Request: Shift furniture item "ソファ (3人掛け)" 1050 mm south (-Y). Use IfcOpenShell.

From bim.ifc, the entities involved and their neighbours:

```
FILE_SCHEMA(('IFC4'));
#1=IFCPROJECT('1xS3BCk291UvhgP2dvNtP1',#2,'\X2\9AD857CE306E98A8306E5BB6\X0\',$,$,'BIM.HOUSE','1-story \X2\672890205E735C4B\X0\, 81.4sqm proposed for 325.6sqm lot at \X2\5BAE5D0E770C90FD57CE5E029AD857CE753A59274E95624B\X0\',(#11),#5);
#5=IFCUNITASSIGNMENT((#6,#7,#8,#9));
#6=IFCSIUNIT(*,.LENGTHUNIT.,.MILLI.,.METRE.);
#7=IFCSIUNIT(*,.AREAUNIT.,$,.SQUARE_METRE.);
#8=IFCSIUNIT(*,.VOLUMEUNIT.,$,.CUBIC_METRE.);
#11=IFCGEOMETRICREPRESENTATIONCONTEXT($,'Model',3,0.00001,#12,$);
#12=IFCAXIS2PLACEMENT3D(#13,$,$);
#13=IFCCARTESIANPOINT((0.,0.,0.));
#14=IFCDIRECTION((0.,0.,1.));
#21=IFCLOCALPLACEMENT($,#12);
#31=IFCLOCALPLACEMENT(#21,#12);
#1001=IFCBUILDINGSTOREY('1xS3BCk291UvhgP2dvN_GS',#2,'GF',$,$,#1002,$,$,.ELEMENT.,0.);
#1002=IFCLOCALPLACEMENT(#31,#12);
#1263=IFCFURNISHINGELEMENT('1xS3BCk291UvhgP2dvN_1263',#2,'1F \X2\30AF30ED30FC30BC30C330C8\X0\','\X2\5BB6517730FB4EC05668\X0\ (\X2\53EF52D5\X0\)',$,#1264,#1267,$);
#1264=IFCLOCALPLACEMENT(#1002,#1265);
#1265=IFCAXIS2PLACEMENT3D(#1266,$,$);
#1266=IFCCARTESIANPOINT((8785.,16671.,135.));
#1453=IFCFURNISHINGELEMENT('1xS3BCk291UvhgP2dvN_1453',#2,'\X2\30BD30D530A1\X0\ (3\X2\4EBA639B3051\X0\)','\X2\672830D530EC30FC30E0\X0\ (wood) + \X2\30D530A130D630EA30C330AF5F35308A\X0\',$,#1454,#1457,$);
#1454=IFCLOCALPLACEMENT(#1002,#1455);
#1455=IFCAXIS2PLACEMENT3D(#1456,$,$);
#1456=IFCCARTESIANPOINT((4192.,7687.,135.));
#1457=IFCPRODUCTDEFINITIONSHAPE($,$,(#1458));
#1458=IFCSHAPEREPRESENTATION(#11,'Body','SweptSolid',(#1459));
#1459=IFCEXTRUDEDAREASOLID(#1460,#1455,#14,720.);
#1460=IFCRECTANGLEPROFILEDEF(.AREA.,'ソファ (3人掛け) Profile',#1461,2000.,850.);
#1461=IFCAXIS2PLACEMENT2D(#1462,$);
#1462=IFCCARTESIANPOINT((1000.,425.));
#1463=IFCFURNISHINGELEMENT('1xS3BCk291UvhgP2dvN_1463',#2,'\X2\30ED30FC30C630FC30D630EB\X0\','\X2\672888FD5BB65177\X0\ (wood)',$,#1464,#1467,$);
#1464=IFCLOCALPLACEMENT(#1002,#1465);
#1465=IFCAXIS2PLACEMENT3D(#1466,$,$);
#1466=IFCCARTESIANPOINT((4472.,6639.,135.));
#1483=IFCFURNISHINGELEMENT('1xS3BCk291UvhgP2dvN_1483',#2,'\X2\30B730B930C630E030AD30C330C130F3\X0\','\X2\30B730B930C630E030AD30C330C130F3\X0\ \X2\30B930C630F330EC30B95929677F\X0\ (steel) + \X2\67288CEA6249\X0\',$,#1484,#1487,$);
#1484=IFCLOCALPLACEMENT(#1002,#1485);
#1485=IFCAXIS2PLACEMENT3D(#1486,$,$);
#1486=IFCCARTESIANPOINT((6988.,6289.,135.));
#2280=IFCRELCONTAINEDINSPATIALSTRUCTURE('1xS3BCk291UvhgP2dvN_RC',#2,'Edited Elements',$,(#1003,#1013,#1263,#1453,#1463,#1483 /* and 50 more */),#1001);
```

```python
import ifcopenshell
import ifcopenshell.api.geometry
import ifcopenshell.util.placement
import ifcopenshell.util.unit

model = ifcopenshell.open("bim.ifc")
unit_scale = ifcopenshell.util.unit.calculate_unit_scale(model)

item = model.by_guid("1xS3BCk291UvhgP2dvN_1453")
matrix = ifcopenshell.util.placement.get_local_placement(item.ObjectPlacement)
matrix[1, 3] -= 1.05 / unit_scale
ifcopenshell.api.geometry.edit_object_placement(model, product=item, matrix=matrix, is_si=False)

print(ifcopenshell.util.placement.get_local_placement(item.ObjectPlacement).round(3) + 0.0)

model.write("bim_v2.ifc")
```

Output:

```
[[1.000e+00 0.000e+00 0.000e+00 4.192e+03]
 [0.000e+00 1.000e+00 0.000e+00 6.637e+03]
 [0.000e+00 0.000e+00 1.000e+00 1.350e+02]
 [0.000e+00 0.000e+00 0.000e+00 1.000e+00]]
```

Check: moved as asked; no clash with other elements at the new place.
